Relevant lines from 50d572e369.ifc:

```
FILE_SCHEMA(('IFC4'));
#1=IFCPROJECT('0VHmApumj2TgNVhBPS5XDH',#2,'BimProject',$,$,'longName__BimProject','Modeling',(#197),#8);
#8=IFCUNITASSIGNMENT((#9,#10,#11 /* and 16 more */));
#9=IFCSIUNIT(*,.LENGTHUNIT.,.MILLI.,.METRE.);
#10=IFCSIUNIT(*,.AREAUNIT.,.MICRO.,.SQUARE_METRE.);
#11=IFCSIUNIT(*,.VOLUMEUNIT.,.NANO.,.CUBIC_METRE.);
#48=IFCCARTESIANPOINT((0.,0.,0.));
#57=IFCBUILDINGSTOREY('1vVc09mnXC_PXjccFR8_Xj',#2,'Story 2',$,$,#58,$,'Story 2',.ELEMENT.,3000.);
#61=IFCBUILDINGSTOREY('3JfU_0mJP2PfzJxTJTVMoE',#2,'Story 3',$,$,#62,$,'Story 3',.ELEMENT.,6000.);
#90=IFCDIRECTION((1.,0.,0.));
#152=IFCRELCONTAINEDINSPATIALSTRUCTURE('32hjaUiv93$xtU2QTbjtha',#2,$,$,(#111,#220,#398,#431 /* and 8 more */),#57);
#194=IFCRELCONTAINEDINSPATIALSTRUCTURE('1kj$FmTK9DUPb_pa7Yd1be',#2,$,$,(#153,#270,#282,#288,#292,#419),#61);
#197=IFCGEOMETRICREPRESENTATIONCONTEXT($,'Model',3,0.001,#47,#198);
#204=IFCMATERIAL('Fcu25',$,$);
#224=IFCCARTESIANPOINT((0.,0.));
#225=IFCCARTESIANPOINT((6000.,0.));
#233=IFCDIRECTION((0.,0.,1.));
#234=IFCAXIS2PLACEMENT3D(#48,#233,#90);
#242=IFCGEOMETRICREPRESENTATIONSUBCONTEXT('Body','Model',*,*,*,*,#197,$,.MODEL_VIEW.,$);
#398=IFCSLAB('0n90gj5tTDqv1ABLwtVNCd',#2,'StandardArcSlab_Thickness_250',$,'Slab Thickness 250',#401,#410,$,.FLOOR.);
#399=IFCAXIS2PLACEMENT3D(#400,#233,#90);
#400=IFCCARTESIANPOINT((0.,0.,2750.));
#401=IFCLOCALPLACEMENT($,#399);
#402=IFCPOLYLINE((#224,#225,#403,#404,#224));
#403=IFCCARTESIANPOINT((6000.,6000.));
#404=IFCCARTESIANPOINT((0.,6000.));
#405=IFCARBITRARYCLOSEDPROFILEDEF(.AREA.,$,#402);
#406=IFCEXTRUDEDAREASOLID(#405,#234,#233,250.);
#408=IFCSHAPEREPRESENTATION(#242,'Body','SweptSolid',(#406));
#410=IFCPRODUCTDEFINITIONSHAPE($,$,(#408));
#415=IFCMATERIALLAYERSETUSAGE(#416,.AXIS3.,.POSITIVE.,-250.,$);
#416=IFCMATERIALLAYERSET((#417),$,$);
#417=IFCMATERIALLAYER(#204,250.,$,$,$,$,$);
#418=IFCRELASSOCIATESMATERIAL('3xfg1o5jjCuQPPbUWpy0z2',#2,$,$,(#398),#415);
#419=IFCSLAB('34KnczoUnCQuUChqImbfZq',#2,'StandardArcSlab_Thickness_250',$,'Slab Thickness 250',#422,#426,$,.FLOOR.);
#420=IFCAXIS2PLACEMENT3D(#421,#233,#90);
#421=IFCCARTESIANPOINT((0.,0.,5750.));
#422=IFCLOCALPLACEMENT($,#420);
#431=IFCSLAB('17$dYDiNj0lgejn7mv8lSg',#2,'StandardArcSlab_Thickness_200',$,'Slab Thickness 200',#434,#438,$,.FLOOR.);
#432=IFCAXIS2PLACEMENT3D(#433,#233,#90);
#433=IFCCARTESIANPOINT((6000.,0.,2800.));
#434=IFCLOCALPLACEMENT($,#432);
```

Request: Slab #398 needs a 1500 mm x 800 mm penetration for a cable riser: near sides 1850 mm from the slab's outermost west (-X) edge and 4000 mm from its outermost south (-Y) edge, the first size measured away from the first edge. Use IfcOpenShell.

```python
import numpy as np
import ifcopenshell
import ifcopenshell.api.feature
import ifcopenshell.api.geometry
import ifcopenshell.api.root
import ifcopenshell.geom
import ifcopenshell.util.placement
import ifcopenshell.util.representation
import ifcopenshell.util.shape
import ifcopenshell.util.unit

model = ifcopenshell.open("50d572e369.ifc")
unit_scale = ifcopenshell.util.unit.calculate_unit_scale(model)
settings = ifcopenshell.geom.settings()


def volume(element):
    """Net volume in cubic metres, openings subtracted."""
    shape = ifcopenshell.geom.create_shape(settings, element)
    return ifcopenshell.util.shape.get_volume(shape.geometry)


slab = model.by_guid("0n90gj5tTDqv1ABLwtVNCd")
before = volume(slab)

# Extent in the slab's own axes, in metres. The edges named are its -X and -Y sides.
slab_shape = ifcopenshell.geom.create_shape(settings, slab)
vertices = ifcopenshell.util.shape.get_vertices(slab_shape.geometry)
x_min, y_min, bottom = vertices.min(axis=0)
top = vertices[:, 2].max()

opening = ifcopenshell.api.root.create_entity(model, ifc_class="IfcOpeningElement", name="Cable riser opening", predefined_type="OPENING")
context = ifcopenshell.util.representation.get_context(model, "Model", "Body", "MODEL_VIEW")
width, depth = 1.5, 0.8
outline = [(0.0, 0.0), (width, 0.0), (width, depth), (0.0, depth), (0.0, 0.0)]
# Overshoot both faces by 50 mm so the cut is clean.
shape = ifcopenshell.api.geometry.add_slab_representation(
    model, context=context, depth=top - bottom + 0.1, polyline=outline
)
ifcopenshell.api.geometry.assign_representation(model, product=opening, representation=shape)

matrix = ifcopenshell.util.placement.get_local_placement(slab.ObjectPlacement)
matrix[:, 3] = matrix @ np.append(np.array([x_min + 1.85, y_min + 4, bottom - 0.05]) / unit_scale, 1.0)
ifcopenshell.api.geometry.edit_object_placement(model, product=opening, matrix=matrix, is_si=False)
ifcopenshell.api.feature.add_feature(model, feature=opening, element=slab)

after = volume(slab)

print(f"slab volume {before:.3f} -> {after:.3f} m3")

model.write("50d572e369_edited.ifc")
```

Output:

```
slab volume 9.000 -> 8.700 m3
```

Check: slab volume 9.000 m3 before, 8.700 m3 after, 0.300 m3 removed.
